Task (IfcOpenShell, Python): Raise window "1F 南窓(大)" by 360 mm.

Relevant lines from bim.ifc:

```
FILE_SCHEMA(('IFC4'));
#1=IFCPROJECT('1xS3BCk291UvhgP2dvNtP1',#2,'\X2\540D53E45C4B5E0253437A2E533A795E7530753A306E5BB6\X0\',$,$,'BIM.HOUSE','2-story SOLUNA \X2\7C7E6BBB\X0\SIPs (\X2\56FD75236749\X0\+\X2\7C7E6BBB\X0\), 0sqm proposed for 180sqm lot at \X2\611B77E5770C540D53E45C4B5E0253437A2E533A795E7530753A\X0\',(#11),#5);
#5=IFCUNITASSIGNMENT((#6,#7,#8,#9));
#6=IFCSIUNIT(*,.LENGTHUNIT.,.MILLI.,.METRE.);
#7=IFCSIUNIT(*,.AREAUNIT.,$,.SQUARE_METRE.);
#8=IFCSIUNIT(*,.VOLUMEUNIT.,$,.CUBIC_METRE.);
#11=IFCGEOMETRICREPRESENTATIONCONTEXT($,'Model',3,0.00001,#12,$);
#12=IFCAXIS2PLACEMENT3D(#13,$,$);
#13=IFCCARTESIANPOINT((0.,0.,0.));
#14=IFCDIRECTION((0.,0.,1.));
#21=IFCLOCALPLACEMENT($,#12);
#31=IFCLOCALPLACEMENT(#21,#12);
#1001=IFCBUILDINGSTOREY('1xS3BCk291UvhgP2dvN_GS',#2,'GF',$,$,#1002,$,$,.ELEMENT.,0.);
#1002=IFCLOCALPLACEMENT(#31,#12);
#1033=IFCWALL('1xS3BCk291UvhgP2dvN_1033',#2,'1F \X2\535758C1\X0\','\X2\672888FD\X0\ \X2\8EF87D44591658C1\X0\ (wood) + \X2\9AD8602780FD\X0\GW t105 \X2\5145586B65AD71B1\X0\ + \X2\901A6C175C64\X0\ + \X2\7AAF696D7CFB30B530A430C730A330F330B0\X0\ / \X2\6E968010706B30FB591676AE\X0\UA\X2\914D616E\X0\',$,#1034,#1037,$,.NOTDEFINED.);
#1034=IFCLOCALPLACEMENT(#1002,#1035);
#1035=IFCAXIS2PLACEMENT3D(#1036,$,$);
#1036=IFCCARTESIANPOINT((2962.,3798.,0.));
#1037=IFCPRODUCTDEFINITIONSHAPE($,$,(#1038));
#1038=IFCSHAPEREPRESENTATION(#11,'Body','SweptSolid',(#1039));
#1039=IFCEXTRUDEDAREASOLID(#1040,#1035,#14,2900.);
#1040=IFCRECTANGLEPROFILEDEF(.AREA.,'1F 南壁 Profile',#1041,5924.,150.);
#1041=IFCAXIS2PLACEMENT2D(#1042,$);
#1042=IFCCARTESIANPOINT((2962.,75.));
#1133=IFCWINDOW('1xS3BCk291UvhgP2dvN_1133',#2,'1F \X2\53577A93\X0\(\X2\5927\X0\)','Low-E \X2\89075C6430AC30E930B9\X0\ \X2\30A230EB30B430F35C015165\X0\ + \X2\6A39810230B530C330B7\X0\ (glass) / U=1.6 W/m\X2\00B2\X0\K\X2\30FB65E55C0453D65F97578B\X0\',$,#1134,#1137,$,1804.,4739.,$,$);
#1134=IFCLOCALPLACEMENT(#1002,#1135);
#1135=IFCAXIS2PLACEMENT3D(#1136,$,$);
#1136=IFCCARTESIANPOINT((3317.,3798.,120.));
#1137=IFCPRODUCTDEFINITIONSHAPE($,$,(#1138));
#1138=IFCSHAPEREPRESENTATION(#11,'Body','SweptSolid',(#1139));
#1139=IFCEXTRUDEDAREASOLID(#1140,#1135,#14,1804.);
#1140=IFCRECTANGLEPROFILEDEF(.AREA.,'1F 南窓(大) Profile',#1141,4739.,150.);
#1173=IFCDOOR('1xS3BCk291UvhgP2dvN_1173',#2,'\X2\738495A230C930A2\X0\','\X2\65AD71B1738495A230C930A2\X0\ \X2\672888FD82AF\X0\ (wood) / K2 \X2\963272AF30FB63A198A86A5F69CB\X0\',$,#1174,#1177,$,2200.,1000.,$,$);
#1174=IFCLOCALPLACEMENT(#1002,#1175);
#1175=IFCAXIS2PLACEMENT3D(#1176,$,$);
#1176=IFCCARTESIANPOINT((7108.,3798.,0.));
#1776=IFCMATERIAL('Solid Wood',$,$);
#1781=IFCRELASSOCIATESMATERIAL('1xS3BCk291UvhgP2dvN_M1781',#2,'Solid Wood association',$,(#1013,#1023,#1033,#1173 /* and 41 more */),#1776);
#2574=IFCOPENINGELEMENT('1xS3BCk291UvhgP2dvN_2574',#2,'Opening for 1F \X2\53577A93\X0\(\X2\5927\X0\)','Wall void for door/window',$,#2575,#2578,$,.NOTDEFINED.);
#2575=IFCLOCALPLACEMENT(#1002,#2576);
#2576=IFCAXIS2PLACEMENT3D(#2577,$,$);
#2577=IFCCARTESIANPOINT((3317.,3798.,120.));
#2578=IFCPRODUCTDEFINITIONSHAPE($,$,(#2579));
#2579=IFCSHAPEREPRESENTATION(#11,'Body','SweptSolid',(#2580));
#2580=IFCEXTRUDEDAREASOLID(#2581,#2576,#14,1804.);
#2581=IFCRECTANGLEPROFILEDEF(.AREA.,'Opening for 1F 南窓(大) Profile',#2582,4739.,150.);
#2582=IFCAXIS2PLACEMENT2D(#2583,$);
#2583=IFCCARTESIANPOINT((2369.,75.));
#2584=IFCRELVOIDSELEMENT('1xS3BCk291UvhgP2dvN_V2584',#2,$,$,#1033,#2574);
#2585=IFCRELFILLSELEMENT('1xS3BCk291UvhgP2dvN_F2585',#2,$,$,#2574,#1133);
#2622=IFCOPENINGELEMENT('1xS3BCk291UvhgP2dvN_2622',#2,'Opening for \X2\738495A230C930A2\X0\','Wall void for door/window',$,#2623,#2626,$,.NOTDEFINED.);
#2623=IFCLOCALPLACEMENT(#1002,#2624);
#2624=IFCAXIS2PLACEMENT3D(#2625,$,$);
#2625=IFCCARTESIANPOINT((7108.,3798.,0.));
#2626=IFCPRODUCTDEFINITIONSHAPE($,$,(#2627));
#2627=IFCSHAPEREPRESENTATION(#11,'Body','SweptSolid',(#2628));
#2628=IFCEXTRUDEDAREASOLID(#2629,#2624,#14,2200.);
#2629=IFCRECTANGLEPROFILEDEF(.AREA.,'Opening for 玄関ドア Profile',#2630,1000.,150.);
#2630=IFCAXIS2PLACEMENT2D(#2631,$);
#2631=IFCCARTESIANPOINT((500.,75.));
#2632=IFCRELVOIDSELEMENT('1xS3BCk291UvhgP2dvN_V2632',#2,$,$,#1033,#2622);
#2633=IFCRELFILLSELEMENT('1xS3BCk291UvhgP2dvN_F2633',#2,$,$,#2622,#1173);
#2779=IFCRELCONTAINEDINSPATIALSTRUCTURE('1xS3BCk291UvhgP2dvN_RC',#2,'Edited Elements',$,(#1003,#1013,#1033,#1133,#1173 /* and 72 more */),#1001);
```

```python
import numpy as np
import ifcopenshell
import ifcopenshell.api.geometry
import ifcopenshell.util.placement
import ifcopenshell.util.unit

model = ifcopenshell.open("bim.ifc")
unit_scale = ifcopenshell.util.unit.calculate_unit_scale(model)

window = model.by_id(1133)
opening = window.FillsVoids[0].RelatingOpeningElement
dz = 0.36 / unit_scale

shift = np.array([0.0, 0.0, dz])
# The window is not placed relative to its opening, so move both.
for product in (opening, window):
    matrix = ifcopenshell.util.placement.get_local_placement(product.ObjectPlacement)
    matrix[:3, 3] += shift
    ifcopenshell.api.geometry.edit_object_placement(model, product=product, matrix=matrix, is_si=False)

print(f"moved by {dz * unit_scale:+.3f} m")

model.write("bim_rev.ifc")
```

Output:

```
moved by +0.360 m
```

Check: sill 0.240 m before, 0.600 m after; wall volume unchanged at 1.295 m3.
